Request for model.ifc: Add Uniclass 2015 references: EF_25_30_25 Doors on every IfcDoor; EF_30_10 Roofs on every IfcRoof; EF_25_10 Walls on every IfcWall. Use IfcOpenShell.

First a look at what the model holds.

```python
import ifcopenshell

model = ifcopenshell.open("model.ifc")
print(model.schema)
print("classifications:", [c.Name for c in model.by_type("IfcClassification")])
for ifc_class in ("IfcDoor", "IfcRoof", "IfcStair", "IfcWall", "IfcWindow"):
    print(ifc_class, len(model.by_type(ifc_class)))
```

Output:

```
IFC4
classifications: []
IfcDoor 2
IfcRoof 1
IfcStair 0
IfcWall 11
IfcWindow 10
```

```python
import ifcopenshell
import ifcopenshell.api.classification

model = ifcopenshell.open("model.ifc")

system = ifcopenshell.api.classification.add_classification(model, classification="Uniclass 2015")

codes = {
    "IfcDoor": ("EF_25_30_25", "Doors"),
    "IfcRoof": ("EF_30_10", "Roofs"),
    "IfcWall": ("EF_25_10", "Walls"),
}
for ifc_class, (code, name) in codes.items():
    products = model.by_type(ifc_class)
    ifcopenshell.api.classification.add_reference(
        model, products=products, classification=system, identification=code, name=name
    )
    print(code, len(products))

model.write("model_edited.ifc")
```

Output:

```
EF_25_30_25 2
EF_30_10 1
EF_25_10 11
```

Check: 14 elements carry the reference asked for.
